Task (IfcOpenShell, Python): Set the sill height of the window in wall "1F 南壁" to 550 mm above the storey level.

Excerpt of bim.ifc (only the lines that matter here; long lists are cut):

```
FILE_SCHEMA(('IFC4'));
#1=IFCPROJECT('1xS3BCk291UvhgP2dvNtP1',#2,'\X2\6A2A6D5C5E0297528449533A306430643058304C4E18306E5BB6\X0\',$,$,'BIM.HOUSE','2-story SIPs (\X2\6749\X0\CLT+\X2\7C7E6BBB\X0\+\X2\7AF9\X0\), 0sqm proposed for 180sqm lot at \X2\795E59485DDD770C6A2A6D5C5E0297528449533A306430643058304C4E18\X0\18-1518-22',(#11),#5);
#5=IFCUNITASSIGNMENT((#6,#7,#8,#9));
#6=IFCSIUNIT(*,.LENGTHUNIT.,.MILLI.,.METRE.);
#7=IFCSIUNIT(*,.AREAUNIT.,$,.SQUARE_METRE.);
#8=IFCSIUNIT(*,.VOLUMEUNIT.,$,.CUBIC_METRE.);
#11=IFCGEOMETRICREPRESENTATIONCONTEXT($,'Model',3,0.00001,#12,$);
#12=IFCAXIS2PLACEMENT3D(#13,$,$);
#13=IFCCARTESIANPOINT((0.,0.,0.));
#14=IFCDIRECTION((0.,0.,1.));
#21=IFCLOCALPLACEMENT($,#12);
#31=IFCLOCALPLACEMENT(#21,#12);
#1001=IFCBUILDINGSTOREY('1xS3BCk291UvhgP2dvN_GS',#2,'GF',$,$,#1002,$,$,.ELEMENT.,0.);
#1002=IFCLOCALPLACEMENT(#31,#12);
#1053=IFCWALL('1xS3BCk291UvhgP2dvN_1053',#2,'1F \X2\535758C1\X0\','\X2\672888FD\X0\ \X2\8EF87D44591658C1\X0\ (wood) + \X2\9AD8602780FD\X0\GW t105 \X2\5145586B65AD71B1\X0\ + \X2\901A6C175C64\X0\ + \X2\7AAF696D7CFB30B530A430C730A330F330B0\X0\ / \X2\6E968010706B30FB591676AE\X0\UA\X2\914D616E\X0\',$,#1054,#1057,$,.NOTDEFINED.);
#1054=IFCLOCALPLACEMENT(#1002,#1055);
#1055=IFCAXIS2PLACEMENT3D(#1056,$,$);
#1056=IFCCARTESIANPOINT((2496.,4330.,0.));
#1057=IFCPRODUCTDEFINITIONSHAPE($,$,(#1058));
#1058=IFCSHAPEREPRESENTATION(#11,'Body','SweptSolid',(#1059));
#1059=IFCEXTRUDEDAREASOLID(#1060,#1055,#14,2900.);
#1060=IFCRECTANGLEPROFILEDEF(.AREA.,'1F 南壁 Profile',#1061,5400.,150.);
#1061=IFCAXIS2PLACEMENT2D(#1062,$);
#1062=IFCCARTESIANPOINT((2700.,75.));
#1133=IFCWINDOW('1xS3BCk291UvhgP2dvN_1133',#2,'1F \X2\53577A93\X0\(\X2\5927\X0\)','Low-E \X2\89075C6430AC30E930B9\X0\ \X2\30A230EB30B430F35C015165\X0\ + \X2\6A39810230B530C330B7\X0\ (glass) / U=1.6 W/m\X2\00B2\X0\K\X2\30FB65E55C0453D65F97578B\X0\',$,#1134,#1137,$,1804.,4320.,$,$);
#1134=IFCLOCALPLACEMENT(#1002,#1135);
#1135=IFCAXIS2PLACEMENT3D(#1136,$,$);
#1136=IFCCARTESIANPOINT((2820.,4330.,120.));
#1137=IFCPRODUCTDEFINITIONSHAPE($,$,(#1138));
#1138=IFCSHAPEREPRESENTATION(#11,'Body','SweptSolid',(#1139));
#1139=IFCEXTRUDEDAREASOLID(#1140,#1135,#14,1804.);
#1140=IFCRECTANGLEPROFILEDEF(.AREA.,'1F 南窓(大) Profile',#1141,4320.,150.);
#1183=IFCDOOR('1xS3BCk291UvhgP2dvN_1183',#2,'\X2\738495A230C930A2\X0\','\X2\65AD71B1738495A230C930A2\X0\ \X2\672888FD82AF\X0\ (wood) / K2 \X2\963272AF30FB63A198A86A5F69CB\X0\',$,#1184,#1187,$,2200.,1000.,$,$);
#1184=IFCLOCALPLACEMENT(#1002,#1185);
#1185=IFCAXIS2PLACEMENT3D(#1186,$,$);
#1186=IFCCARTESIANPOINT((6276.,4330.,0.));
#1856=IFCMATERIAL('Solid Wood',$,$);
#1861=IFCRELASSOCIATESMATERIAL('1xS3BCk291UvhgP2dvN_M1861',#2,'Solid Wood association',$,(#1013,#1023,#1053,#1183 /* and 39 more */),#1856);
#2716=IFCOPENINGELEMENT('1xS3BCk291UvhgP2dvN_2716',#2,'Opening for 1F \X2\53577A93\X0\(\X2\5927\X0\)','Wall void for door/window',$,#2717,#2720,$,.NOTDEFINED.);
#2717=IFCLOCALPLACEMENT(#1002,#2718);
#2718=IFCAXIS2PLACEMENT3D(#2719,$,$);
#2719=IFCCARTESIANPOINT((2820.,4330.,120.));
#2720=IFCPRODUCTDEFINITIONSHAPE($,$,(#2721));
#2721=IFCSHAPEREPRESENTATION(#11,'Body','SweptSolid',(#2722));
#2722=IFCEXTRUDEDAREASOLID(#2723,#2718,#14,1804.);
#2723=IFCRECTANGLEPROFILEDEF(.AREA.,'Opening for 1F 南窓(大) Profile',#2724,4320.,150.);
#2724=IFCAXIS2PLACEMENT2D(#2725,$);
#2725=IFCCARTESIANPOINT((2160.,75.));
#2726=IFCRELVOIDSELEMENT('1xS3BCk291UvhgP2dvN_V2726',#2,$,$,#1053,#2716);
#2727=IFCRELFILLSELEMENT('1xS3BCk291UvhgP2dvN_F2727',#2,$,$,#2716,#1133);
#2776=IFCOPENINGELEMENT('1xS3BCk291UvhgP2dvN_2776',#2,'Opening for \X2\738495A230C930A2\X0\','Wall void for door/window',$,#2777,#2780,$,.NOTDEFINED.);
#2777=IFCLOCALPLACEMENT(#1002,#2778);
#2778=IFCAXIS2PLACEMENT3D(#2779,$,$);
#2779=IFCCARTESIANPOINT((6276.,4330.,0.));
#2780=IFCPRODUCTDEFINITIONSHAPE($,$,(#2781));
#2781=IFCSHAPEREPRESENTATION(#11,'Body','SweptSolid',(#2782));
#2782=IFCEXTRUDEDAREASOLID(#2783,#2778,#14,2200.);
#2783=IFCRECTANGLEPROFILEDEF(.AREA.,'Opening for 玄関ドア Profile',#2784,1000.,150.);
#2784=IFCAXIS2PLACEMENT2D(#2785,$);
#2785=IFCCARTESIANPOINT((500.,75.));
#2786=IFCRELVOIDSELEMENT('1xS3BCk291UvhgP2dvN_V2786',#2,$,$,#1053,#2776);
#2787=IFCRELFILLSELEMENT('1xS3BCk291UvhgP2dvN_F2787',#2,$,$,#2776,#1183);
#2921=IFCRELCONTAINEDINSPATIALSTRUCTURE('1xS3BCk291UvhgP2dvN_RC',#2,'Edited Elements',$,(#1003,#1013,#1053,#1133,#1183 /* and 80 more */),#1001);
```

```python
import numpy as np
import ifcopenshell
import ifcopenshell.api.geometry
import ifcopenshell.geom
import ifcopenshell.util.element
import ifcopenshell.util.placement
import ifcopenshell.util.shape
import ifcopenshell.util.unit

model = ifcopenshell.open("bim.ifc")
unit_scale = ifcopenshell.util.unit.calculate_unit_scale(model)

window = model.by_guid("1xS3BCk291UvhgP2dvN_1133")
opening = window.FillsVoids[0].RelatingOpeningElement
storey = ifcopenshell.util.element.get_container(window, ifc_class="IfcBuildingStorey")
level = ifcopenshell.util.placement.get_local_placement(storey.ObjectPlacement)[2, 3]

# The opening's origin need not be at the sill, so measure its lowest point.
shape = ifcopenshell.geom.create_shape(ifcopenshell.geom.settings(), opening)
bottom = ifcopenshell.util.shape.get_shape_bottom_elevation(shape, shape.geometry) / unit_scale
dz = level + 550.0 - bottom

shift = np.array([0.0, 0.0, dz])
# The window is not placed relative to its opening, so move both.
for product in (opening, window):
    matrix = ifcopenshell.util.placement.get_local_placement(product.ObjectPlacement)
    matrix[:3, 3] += shift
    ifcopenshell.api.geometry.edit_object_placement(model, product=product, matrix=matrix, is_si=False)

print(f"moved by {dz * unit_scale:+.3f} m")

model.write("bim_edited.ifc")
```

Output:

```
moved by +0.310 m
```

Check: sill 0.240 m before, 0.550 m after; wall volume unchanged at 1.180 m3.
